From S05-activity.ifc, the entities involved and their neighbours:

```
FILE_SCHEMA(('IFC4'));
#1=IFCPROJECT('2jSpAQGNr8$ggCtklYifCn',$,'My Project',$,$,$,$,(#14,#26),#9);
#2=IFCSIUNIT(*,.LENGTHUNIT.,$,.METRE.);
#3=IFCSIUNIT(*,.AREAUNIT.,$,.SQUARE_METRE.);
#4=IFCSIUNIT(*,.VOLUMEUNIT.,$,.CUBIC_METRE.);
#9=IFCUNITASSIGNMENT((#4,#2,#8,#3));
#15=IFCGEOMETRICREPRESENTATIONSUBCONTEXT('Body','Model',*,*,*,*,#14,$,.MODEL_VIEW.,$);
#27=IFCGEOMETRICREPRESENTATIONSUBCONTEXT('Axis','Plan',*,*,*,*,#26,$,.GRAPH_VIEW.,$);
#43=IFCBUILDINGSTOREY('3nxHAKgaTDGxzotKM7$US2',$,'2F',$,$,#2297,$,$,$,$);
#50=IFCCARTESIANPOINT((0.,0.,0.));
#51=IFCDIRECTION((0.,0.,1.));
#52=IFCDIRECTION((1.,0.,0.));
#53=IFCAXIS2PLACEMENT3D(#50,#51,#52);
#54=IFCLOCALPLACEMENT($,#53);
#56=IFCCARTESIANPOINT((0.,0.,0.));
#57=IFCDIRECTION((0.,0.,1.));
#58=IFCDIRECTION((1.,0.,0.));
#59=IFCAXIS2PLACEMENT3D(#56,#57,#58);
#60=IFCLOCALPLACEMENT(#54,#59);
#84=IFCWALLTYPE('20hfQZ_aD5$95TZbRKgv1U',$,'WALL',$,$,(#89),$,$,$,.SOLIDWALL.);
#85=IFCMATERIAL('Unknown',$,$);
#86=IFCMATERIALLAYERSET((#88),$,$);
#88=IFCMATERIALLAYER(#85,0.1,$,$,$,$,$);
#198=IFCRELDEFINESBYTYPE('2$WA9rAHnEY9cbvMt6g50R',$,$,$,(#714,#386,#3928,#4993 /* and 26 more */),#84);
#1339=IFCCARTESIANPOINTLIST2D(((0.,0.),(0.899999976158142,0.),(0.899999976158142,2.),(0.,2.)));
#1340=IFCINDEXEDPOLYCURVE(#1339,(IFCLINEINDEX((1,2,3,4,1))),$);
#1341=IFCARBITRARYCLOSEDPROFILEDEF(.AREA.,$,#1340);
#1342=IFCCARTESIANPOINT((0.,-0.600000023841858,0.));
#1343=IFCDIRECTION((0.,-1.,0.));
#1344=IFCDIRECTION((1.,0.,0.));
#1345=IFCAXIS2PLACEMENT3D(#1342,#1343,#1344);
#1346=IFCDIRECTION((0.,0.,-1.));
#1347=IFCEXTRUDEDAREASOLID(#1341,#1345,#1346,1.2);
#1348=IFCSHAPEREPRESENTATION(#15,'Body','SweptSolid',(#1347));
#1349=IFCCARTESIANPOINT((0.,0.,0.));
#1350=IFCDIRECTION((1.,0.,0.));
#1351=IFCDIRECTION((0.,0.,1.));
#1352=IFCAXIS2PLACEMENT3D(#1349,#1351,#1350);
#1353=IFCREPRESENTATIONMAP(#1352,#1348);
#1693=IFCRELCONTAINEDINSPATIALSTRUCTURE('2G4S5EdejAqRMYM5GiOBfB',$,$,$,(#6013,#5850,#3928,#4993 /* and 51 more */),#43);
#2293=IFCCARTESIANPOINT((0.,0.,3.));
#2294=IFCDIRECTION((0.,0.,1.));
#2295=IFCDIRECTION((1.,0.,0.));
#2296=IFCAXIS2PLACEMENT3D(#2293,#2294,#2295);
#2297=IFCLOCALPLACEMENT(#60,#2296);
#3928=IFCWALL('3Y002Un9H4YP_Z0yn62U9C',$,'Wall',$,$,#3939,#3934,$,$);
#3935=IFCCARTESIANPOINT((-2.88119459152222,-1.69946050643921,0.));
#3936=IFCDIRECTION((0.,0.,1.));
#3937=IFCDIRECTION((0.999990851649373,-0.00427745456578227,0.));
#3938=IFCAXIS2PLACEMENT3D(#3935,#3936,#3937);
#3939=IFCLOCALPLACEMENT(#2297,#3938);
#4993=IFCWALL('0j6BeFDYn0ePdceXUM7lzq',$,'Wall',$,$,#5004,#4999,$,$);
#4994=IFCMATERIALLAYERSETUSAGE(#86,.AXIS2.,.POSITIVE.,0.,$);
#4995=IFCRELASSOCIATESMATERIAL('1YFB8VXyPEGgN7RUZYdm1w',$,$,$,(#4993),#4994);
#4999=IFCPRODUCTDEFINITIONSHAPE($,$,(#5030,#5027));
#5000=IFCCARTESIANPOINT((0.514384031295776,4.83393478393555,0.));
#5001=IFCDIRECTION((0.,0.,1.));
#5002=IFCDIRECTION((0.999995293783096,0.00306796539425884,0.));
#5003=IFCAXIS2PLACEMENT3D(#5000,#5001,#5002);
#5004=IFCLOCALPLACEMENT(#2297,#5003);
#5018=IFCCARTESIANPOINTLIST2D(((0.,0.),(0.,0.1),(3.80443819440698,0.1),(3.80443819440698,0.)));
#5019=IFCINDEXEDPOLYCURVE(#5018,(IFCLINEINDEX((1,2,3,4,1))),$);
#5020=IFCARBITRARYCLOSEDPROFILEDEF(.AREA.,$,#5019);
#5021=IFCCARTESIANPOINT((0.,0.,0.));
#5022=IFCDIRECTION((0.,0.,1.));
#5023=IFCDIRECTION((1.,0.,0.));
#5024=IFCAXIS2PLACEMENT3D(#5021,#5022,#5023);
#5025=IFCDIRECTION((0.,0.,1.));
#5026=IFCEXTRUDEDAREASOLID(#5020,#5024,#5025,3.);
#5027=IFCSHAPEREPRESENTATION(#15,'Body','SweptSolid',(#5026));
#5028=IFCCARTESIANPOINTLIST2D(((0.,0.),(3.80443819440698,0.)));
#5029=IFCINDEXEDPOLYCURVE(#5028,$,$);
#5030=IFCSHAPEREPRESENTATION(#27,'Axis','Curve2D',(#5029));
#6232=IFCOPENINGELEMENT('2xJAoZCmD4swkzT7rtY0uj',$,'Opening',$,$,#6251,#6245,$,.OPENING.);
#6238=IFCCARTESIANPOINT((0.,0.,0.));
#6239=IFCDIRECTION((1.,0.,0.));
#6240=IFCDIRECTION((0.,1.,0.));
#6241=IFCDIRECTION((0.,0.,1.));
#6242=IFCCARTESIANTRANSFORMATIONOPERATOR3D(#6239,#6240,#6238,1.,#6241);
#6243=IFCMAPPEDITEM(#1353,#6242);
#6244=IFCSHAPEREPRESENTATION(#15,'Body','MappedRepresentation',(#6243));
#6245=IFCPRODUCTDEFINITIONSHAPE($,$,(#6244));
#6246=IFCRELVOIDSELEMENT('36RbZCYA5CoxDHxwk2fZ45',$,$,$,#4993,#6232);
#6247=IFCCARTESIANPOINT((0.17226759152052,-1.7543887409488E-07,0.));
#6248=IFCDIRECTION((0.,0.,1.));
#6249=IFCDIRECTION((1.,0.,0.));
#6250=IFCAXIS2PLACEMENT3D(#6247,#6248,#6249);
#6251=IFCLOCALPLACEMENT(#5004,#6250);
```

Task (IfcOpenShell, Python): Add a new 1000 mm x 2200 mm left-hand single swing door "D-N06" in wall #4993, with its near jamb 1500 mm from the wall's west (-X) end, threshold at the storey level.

```python
import numpy as np
import ifcopenshell
import ifcopenshell.api.feature
import ifcopenshell.api.geometry
import ifcopenshell.api.root
import ifcopenshell.api.spatial
import ifcopenshell.geom
import ifcopenshell.util.element
import ifcopenshell.util.placement
import ifcopenshell.util.representation
import ifcopenshell.util.shape
import ifcopenshell.util.unit

model = ifcopenshell.open("S05-activity.ifc")
unit_scale = ifcopenshell.util.unit.calculate_unit_scale(model)
settings = ifcopenshell.geom.settings()


def volume(element):
    """Net volume in cubic metres, openings subtracted."""
    shape = ifcopenshell.geom.create_shape(settings, element)
    return ifcopenshell.util.shape.get_volume(shape.geometry)


wall = model.by_id(4993)
storey = ifcopenshell.util.element.get_container(wall, ifc_class="IfcBuildingStorey")
context = ifcopenshell.util.representation.get_context(model, "Model", "Body", "MODEL_VIEW")
before = volume(wall)

width, height, from_end, sill = 1, 2.2, 1.5, 0.0  # metres

# The wall runs along its own X axis, and the end named is its -X end.
wall_shape = ifcopenshell.geom.create_shape(settings, wall)
x, y, z = ifcopenshell.util.shape.get_vertices(wall_shape.geometry).T
start = x.min() + from_end
face, thickness = float(y.min()), float(y.max() - y.min())
wall_matrix = ifcopenshell.util.placement.get_local_placement(wall.ObjectPlacement)
level = ifcopenshell.util.placement.get_local_placement(storey.ObjectPlacement)[2, 3]


def in_wall(x, y):
    """Placement at x, y metres in the wall's axes, at sill height."""
    matrix = wall_matrix.copy()
    matrix[:, 3] = wall_matrix @ np.array([x / unit_scale, y / unit_scale, 0.0, 1.0])
    matrix[2, 3] = level + sill / unit_scale
    return matrix


# Opening: a box that overshoots both wall faces by 50 mm.
opening = ifcopenshell.api.root.create_entity(model, ifc_class="IfcOpeningElement", predefined_type="OPENING")
box = ifcopenshell.api.geometry.add_wall_representation(
    model, context=context, length=width, height=height, thickness=thickness + 0.1
)
ifcopenshell.api.geometry.assign_representation(model, product=opening, representation=box)
ifcopenshell.api.geometry.edit_object_placement(model, product=opening, matrix=in_wall(start, face - 0.05), is_si=False)
ifcopenshell.api.feature.add_feature(model, feature=opening, element=wall)

door = ifcopenshell.api.root.create_entity(model, ifc_class="IfcDoor", name="D-N06", predefined_type="DOOR")
door.OverallWidth, door.OverallHeight = width / unit_scale, height / unit_scale
door.OperationType = "SINGLE_SWING_LEFT"
body = ifcopenshell.api.geometry.add_door_representation(
    model,
    context=context,
    overall_width=door.OverallWidth,
    overall_height=door.OverallHeight,
    operation_type="SINGLE_SWING_LEFT",
    lining_properties={"LiningDepth": thickness / unit_scale, "ThresholdDepth": thickness / unit_scale},
)
ifcopenshell.api.geometry.assign_representation(model, product=door, representation=body)
ifcopenshell.api.spatial.assign_container(model, products=[door], relating_structure=storey)
ifcopenshell.api.feature.add_filling(model, opening=opening, element=door)

# The lining spans the wall, so the door starts at the wall face.
ifcopenshell.api.geometry.edit_object_placement(model, product=door, matrix=in_wall(start, face), is_si=False)

after = volume(wall)

print(f"wall volume {before:.3f} -> {after:.3f} m3")

model.write("S05-activity_edited.ifc")
```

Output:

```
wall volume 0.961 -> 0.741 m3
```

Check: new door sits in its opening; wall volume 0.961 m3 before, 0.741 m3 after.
